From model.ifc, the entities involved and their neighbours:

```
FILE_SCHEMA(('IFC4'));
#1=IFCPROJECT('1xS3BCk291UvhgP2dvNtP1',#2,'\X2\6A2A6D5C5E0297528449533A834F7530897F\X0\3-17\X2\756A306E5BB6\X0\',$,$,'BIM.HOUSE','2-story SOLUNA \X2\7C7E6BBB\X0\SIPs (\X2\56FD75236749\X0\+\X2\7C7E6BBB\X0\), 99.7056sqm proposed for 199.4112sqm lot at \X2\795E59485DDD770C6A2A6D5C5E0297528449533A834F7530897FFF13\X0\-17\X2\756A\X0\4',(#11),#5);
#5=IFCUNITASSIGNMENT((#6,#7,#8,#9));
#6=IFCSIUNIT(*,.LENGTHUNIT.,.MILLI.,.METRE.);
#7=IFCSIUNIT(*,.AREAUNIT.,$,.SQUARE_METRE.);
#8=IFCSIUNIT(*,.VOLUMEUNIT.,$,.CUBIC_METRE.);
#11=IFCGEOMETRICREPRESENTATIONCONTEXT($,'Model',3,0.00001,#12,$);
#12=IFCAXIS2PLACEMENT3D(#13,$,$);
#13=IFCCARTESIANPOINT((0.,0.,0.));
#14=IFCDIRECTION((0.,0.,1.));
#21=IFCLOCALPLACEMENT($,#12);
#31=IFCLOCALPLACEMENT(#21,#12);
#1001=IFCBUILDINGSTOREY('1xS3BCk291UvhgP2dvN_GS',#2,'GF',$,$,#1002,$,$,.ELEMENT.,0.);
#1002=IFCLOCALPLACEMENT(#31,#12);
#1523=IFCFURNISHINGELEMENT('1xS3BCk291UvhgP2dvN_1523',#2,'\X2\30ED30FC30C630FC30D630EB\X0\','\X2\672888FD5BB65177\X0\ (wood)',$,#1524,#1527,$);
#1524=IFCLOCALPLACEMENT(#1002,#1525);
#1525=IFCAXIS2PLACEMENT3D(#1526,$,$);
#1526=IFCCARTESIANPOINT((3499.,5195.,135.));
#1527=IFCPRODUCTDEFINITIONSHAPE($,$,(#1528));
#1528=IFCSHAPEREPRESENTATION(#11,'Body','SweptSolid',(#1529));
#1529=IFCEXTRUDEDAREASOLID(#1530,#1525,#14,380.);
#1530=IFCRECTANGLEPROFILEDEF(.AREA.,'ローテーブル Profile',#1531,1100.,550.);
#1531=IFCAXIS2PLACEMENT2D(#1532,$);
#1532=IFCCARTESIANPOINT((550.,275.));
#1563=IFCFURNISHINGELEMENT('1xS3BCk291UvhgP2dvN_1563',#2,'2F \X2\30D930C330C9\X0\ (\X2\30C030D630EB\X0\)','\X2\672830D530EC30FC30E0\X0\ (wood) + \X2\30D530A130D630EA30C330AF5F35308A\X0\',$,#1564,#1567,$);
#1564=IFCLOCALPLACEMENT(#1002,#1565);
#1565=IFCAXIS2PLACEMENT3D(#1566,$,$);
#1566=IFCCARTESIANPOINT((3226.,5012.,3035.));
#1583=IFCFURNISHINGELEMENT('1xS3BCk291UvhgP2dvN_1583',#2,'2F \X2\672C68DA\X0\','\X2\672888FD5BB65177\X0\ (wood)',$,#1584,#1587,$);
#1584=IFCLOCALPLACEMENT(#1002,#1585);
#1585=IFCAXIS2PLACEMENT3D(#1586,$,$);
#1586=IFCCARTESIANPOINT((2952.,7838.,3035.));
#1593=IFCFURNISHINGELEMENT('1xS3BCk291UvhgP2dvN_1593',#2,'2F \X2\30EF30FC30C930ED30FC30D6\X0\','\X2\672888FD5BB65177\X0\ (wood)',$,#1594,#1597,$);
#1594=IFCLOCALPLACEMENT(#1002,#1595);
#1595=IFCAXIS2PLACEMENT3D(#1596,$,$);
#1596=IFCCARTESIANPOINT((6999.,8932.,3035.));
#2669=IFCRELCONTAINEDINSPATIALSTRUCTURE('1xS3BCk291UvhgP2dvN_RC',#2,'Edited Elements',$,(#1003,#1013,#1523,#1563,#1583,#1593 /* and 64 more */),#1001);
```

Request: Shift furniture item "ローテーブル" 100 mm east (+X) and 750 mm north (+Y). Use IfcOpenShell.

```python
import ifcopenshell
import ifcopenshell.api.geometry
import ifcopenshell.util.placement
import ifcopenshell.util.unit

model = ifcopenshell.open("model.ifc")
unit_scale = ifcopenshell.util.unit.calculate_unit_scale(model)

item = model.by_guid("1xS3BCk291UvhgP2dvN_1523")
matrix = ifcopenshell.util.placement.get_local_placement(item.ObjectPlacement)
matrix[0, 3] += 0.1 / unit_scale
matrix[1, 3] += 0.75 / unit_scale
ifcopenshell.api.geometry.edit_object_placement(model, product=item, matrix=matrix, is_si=False)

print(ifcopenshell.util.placement.get_local_placement(item.ObjectPlacement).round(3) + 0.0)

model.write("model-out.ifc")
```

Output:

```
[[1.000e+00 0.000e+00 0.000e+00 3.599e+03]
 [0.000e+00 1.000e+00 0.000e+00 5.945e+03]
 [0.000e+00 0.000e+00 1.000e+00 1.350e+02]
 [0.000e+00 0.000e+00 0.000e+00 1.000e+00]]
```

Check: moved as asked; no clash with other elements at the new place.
